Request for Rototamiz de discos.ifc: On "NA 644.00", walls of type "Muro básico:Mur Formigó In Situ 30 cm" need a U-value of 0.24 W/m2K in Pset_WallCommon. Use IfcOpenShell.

First a look at what the model holds.

```python
import ifcopenshell
import ifcopenshell.util.element

model = ifcopenshell.open("Rototamiz de discos.ifc")
print(model.schema)
storey = next(s for s in model.by_type("IfcBuildingStorey") if s.Name == "NA 644.00")
walls = [e for e in ifcopenshell.util.element.get_decomposition(storey) if e.is_a("IfcWall")]
seen = {}
for e in walls:
    element_type = ifcopenshell.util.element.get_type(e)
    key = (element_type.Name if element_type != e and element_type else None, ifcopenshell.util.element.get_pset(e, "Pset_WallCommon", "ThermalTransmittance"))
    seen[key] = seen.get(key, 0) + 1
for (name, value), count in sorted(seen.items(), key=str):
    print(count, "x", name, "|", value)
```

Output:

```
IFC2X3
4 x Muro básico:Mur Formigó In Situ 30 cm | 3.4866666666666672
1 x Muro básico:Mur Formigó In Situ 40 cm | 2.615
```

```python
import ifcopenshell
import ifcopenshell.api.pset
import ifcopenshell.util.element

model = ifcopenshell.open("Rototamiz de discos.ifc")

storey = next(s for s in model.by_type("IfcBuildingStorey") if s.Name == "NA 644.00")
walls = [e for e in ifcopenshell.util.element.get_decomposition(storey) if e.is_a("IfcWall")]

count = 0
for e in walls:
    element_type = ifcopenshell.util.element.get_type(e)
    if element_type in (None, e) or element_type.Name != "Muro básico:Mur Formigó In Situ 30 cm":
        continue
    # add_pset returns the element's existing set when there is one.
    pset = ifcopenshell.api.pset.add_pset(model, product=e, name="Pset_WallCommon")
    ifcopenshell.api.pset.edit_pset(model, pset=pset, properties={"ThermalTransmittance": 0.24})
    count += 1

print(count, "walls updated")

model.write("Rototamiz de discos-out.ifc")
```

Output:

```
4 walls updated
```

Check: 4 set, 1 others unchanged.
